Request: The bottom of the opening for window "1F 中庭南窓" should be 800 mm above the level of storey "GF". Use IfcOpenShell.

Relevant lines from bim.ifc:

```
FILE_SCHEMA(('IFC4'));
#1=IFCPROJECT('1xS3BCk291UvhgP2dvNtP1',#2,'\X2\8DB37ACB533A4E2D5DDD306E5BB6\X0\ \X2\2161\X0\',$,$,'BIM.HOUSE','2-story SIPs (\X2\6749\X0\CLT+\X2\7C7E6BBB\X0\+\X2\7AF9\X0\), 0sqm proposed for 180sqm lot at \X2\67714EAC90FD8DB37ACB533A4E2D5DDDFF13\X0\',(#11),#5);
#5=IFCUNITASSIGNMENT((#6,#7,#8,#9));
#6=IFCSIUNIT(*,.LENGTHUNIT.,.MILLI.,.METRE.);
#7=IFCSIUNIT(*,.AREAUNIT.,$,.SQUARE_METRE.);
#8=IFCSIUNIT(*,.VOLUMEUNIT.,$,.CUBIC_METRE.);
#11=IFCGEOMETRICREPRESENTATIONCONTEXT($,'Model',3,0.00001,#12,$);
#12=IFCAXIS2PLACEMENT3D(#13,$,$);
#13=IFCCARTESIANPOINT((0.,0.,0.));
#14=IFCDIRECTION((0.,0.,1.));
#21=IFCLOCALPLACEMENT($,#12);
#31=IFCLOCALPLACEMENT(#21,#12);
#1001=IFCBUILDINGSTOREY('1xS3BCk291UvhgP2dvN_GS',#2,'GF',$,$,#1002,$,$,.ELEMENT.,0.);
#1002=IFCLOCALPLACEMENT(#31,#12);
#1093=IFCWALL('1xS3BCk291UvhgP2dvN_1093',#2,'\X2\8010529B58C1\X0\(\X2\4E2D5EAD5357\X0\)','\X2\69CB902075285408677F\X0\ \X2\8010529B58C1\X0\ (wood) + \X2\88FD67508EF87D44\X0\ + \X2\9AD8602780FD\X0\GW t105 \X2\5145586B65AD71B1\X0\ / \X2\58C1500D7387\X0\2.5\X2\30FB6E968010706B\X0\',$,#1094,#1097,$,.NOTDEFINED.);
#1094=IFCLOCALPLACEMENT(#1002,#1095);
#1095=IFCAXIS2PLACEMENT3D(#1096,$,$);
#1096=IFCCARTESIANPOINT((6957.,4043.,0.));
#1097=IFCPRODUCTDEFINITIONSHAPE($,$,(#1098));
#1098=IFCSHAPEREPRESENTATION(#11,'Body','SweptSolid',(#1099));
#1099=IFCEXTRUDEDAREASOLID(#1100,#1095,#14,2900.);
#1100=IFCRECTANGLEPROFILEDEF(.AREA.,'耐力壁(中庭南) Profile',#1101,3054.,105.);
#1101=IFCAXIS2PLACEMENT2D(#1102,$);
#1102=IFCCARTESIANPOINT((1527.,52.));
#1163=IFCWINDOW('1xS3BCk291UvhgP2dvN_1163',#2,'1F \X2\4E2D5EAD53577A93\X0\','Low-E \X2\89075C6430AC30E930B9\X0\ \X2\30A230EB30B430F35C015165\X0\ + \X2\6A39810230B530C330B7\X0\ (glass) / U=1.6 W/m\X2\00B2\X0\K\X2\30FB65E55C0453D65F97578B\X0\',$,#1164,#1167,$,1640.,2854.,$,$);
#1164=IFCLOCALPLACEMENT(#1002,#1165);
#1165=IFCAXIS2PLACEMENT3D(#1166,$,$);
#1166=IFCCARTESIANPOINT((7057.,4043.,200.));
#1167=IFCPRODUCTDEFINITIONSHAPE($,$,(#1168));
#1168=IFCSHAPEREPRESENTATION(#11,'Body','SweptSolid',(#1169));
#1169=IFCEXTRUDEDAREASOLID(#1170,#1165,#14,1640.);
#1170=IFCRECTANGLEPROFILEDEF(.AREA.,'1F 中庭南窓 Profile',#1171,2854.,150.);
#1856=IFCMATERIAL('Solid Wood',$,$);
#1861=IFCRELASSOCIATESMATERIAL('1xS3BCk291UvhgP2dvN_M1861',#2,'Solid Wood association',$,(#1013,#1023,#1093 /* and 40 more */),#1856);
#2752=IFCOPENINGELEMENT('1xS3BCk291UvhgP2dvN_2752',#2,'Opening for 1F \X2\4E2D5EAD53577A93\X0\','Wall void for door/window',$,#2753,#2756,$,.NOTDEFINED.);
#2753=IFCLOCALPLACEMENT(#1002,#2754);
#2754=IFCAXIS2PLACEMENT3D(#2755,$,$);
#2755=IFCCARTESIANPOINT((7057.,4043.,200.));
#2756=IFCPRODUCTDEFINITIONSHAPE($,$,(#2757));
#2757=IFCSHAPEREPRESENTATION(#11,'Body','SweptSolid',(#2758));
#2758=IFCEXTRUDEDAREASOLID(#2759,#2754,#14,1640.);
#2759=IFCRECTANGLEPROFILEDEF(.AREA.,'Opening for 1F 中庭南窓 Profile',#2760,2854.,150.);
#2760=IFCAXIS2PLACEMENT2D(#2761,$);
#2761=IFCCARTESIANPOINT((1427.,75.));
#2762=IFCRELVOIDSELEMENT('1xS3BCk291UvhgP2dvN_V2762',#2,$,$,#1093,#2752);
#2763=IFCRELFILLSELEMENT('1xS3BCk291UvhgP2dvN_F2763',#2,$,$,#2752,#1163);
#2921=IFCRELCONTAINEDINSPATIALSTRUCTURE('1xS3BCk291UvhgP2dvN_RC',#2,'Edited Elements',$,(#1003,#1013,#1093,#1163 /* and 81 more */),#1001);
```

```python
import numpy as np
import ifcopenshell
import ifcopenshell.api.geometry
import ifcopenshell.geom
import ifcopenshell.util.element
import ifcopenshell.util.placement
import ifcopenshell.util.shape
import ifcopenshell.util.unit

model = ifcopenshell.open("bim.ifc")
unit_scale = ifcopenshell.util.unit.calculate_unit_scale(model)

window = model.by_guid("1xS3BCk291UvhgP2dvN_1163")
opening = window.FillsVoids[0].RelatingOpeningElement
storey = ifcopenshell.util.element.get_container(window, ifc_class="IfcBuildingStorey")
level = ifcopenshell.util.placement.get_local_placement(storey.ObjectPlacement)[2, 3]

# The opening's origin need not be at the sill, so measure its lowest point.
shape = ifcopenshell.geom.create_shape(ifcopenshell.geom.settings(), opening)
bottom = ifcopenshell.util.shape.get_shape_bottom_elevation(shape, shape.geometry) / unit_scale
dz = level + 0.8 / unit_scale - bottom

shift = np.array([0.0, 0.0, dz])
# The window is not placed relative to its opening, so move both.
for product in (opening, window):
    matrix = ifcopenshell.util.placement.get_local_placement(product.ObjectPlacement)
    matrix[:3, 3] += shift
    ifcopenshell.api.geometry.edit_object_placement(model, product=product, matrix=matrix, is_si=False)

print(f"moved by {dz * unit_scale:+.3f} m")

model.write("bim_edited.ifc")
```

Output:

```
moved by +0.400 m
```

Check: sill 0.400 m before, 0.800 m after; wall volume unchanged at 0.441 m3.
